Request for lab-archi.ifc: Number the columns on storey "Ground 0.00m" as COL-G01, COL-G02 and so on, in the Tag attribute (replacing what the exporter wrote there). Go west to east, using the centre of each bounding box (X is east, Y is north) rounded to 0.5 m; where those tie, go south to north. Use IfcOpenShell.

First a look at what the model holds.

```python
import ifcopenshell
import ifcopenshell.util.element
import ifcopenshell.util.placement

model = ifcopenshell.open("lab-archi.ifc")
print(model.schema)
storey = next(s for s in model.by_type("IfcBuildingStorey") if s.Name == "Ground 0.00m")
columns = [e for e in ifcopenshell.util.element.get_decomposition(storey) if e.is_a("IfcColumn")]
for e in sorted(columns, key=lambda e: e.id()):
    origin = ifcopenshell.util.placement.get_local_placement(e.ObjectPlacement)[:3, 3]
    print(e.id(), e.Tag, e.Name, origin.round(2) + 0.0, sep=" | ")
```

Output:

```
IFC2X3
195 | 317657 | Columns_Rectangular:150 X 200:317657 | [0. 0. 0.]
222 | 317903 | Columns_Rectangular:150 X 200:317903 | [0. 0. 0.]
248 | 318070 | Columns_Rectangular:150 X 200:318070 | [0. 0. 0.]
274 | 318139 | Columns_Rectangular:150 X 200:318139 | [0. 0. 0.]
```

```python
import ifcopenshell
import ifcopenshell.geom
import ifcopenshell.util.element
import ifcopenshell.util.shape

model = ifcopenshell.open("lab-archi.ifc")
settings = ifcopenshell.geom.settings()
settings.set("use-world-coords", True)


def centre(element):
    shape = ifcopenshell.geom.create_shape(settings, element)
    return ifcopenshell.util.shape.get_bbox_centroid(shape.geometry)


storey = next(s for s in model.by_type("IfcBuildingStorey") if s.Name == "Ground 0.00m")
columns = [e for e in ifcopenshell.util.element.get_decomposition(storey) if e.is_a("IfcColumn")]

# Insertion points can sit at a corner or the storey origin, so sort by the geometry (in metres).
centres = {e: centre(e) for e in columns}
columns.sort(key=lambda e: (round(centres[e][0] / 0.5), centres[e][1]))

for i, e in enumerate(columns, start=1):
    number = f"COL-G{i:02d}"
    e.Tag = number
    print(e.id(), number)

model.write("lab-archi_edited.ifc")
```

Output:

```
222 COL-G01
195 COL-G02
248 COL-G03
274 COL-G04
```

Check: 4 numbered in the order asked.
